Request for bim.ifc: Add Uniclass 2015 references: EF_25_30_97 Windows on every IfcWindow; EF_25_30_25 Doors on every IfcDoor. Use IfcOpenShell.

First a look at what the model holds.

```python
import ifcopenshell

model = ifcopenshell.open("bim.ifc")
print(model.schema)
print("classifications:", [c.Name for c in model.by_type("IfcClassification")])
for ifc_class in ("IfcDoor", "IfcRoof", "IfcStair", "IfcWall", "IfcWindow"):
    print(ifc_class, len(model.by_type(ifc_class)))
```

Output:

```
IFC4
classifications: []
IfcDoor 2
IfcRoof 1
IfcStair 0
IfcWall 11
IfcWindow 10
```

```python
import ifcopenshell
import ifcopenshell.api.classification

model = ifcopenshell.open("bim.ifc")

system = ifcopenshell.api.classification.add_classification(model, classification="Uniclass 2015")

codes = {
    "IfcWindow": ("EF_25_30_97", "Windows"),
    "IfcDoor": ("EF_25_30_25", "Doors"),
}
for ifc_class, (code, name) in codes.items():
    products = model.by_type(ifc_class)
    ifcopenshell.api.classification.add_reference(
        model, products=products, classification=system, identification=code, name=name
    )
    print(code, len(products))

model.write("bim_v2.ifc")
```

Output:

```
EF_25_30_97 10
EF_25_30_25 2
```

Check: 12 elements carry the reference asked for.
